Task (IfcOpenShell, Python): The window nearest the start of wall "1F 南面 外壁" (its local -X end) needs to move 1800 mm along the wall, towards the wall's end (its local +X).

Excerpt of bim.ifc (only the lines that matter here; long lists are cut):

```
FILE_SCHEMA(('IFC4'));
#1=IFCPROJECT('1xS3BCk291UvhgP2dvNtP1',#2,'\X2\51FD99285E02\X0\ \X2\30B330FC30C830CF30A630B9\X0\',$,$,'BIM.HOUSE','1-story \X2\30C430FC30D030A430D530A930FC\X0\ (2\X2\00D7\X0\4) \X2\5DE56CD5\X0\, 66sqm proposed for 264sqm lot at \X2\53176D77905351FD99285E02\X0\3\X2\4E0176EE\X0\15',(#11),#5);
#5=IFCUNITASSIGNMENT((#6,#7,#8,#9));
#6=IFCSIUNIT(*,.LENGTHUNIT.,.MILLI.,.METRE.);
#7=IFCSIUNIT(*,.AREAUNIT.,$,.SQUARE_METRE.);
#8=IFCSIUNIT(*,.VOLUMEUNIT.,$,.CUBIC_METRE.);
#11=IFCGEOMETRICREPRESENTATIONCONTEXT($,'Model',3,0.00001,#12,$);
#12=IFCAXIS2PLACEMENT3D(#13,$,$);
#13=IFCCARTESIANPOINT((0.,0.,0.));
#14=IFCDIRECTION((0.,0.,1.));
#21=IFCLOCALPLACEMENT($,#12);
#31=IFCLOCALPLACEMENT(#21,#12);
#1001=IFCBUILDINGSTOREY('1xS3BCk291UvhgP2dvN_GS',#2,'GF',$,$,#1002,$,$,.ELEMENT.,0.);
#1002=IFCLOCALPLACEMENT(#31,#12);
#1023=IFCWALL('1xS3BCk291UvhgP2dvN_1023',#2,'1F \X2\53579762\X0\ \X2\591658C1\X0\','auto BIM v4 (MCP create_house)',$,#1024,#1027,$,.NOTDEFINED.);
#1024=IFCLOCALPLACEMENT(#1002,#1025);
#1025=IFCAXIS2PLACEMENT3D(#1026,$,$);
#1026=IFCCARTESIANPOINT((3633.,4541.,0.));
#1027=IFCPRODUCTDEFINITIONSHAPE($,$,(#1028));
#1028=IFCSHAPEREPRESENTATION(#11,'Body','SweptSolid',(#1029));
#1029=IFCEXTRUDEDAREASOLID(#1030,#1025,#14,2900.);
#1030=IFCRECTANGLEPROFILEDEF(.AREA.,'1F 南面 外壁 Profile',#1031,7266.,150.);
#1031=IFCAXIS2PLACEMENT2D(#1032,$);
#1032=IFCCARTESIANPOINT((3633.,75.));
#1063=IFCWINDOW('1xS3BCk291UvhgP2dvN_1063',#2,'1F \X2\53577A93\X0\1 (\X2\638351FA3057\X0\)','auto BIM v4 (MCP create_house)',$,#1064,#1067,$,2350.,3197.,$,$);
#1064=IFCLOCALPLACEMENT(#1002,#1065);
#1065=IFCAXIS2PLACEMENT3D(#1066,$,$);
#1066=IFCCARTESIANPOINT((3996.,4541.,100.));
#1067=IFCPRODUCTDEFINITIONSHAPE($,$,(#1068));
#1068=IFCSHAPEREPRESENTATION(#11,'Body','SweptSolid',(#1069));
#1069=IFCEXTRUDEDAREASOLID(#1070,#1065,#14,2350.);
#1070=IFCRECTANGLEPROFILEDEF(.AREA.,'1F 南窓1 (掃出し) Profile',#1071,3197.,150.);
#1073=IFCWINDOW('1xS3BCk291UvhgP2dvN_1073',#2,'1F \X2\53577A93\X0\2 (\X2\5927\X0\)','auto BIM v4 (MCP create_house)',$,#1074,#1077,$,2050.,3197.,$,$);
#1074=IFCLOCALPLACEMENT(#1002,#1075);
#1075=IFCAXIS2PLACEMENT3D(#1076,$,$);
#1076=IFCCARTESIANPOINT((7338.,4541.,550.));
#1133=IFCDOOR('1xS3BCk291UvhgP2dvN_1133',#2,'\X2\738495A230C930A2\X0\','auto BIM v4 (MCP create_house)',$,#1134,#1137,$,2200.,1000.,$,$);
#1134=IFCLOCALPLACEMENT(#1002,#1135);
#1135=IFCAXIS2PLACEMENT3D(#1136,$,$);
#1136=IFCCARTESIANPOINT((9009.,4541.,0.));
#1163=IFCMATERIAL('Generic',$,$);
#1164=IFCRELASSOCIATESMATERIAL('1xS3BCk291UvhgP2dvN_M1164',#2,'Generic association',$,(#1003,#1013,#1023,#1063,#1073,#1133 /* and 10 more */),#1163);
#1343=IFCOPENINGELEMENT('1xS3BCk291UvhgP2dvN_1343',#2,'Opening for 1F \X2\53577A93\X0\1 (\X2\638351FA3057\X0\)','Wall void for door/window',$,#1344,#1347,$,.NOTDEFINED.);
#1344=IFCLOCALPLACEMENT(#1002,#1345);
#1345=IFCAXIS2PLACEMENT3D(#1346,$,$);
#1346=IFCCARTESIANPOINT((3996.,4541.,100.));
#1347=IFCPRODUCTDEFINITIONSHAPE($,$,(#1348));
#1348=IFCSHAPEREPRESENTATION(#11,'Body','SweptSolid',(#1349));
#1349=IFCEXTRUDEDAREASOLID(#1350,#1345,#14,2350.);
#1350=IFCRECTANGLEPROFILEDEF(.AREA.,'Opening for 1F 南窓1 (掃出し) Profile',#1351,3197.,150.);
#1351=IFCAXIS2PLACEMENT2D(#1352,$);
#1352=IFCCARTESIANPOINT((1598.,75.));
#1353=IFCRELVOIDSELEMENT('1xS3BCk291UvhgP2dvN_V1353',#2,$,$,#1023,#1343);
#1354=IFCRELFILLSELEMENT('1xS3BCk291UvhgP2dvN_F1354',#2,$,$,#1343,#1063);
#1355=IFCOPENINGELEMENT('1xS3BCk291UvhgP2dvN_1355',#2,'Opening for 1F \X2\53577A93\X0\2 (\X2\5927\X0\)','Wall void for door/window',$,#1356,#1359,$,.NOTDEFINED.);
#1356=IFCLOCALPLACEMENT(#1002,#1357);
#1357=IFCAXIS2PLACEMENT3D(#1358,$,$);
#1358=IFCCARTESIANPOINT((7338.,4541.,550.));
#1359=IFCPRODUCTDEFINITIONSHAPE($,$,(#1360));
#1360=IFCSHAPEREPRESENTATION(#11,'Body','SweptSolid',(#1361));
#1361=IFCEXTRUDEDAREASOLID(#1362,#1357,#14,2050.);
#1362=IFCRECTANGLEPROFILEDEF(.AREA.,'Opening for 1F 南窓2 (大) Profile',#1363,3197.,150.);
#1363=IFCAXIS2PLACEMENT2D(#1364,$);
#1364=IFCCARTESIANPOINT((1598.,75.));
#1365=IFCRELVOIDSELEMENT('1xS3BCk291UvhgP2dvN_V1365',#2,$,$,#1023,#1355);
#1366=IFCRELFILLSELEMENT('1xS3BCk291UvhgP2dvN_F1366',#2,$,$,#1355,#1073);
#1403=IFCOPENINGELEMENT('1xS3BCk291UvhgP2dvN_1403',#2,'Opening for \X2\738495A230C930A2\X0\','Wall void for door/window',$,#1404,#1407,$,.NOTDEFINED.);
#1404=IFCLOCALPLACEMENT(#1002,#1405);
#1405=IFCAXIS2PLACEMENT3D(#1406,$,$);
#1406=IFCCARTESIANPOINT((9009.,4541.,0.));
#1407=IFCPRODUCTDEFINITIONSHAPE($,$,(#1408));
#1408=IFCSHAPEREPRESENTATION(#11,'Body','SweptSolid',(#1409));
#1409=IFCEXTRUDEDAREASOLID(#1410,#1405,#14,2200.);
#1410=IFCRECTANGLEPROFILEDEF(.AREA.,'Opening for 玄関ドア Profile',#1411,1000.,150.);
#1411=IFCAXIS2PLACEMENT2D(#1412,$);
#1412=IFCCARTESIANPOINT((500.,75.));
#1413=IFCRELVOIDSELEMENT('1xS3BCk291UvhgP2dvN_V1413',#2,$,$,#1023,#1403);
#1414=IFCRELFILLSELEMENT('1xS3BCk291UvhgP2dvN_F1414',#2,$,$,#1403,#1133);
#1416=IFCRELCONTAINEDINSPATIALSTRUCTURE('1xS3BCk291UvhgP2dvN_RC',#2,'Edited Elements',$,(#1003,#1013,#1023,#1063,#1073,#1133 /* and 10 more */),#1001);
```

```python
import ifcopenshell
import ifcopenshell.api.geometry
import ifcopenshell.util.placement

model = ifcopenshell.open("bim.ifc")

window = model.by_guid("1xS3BCk291UvhgP2dvN_1063")
opening = window.FillsVoids[0].RelatingOpeningElement
wall = opening.VoidsElements[0].RelatingBuildingElement

wall_matrix = ifcopenshell.util.placement.get_local_placement(wall.ObjectPlacement)
shift = wall_matrix[:3, 0] * 1800.0
before = ifcopenshell.util.placement.get_local_placement(window.ObjectPlacement)[:3, 3].copy()

# The window is not placed relative to its opening, so move both.
for product in (opening, window):
    matrix = ifcopenshell.util.placement.get_local_placement(product.ObjectPlacement)
    matrix[:3, 3] += shift
    ifcopenshell.api.geometry.edit_object_placement(model, product=product, matrix=matrix, is_si=False)

after = ifcopenshell.util.placement.get_local_placement(window.ObjectPlacement)[:3, 3]
print("window moved by", (after - before).round(3) + 0.0)

model.write("bim_rev.ifc")
```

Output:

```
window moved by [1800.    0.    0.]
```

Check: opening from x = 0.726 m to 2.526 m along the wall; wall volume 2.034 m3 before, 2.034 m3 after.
